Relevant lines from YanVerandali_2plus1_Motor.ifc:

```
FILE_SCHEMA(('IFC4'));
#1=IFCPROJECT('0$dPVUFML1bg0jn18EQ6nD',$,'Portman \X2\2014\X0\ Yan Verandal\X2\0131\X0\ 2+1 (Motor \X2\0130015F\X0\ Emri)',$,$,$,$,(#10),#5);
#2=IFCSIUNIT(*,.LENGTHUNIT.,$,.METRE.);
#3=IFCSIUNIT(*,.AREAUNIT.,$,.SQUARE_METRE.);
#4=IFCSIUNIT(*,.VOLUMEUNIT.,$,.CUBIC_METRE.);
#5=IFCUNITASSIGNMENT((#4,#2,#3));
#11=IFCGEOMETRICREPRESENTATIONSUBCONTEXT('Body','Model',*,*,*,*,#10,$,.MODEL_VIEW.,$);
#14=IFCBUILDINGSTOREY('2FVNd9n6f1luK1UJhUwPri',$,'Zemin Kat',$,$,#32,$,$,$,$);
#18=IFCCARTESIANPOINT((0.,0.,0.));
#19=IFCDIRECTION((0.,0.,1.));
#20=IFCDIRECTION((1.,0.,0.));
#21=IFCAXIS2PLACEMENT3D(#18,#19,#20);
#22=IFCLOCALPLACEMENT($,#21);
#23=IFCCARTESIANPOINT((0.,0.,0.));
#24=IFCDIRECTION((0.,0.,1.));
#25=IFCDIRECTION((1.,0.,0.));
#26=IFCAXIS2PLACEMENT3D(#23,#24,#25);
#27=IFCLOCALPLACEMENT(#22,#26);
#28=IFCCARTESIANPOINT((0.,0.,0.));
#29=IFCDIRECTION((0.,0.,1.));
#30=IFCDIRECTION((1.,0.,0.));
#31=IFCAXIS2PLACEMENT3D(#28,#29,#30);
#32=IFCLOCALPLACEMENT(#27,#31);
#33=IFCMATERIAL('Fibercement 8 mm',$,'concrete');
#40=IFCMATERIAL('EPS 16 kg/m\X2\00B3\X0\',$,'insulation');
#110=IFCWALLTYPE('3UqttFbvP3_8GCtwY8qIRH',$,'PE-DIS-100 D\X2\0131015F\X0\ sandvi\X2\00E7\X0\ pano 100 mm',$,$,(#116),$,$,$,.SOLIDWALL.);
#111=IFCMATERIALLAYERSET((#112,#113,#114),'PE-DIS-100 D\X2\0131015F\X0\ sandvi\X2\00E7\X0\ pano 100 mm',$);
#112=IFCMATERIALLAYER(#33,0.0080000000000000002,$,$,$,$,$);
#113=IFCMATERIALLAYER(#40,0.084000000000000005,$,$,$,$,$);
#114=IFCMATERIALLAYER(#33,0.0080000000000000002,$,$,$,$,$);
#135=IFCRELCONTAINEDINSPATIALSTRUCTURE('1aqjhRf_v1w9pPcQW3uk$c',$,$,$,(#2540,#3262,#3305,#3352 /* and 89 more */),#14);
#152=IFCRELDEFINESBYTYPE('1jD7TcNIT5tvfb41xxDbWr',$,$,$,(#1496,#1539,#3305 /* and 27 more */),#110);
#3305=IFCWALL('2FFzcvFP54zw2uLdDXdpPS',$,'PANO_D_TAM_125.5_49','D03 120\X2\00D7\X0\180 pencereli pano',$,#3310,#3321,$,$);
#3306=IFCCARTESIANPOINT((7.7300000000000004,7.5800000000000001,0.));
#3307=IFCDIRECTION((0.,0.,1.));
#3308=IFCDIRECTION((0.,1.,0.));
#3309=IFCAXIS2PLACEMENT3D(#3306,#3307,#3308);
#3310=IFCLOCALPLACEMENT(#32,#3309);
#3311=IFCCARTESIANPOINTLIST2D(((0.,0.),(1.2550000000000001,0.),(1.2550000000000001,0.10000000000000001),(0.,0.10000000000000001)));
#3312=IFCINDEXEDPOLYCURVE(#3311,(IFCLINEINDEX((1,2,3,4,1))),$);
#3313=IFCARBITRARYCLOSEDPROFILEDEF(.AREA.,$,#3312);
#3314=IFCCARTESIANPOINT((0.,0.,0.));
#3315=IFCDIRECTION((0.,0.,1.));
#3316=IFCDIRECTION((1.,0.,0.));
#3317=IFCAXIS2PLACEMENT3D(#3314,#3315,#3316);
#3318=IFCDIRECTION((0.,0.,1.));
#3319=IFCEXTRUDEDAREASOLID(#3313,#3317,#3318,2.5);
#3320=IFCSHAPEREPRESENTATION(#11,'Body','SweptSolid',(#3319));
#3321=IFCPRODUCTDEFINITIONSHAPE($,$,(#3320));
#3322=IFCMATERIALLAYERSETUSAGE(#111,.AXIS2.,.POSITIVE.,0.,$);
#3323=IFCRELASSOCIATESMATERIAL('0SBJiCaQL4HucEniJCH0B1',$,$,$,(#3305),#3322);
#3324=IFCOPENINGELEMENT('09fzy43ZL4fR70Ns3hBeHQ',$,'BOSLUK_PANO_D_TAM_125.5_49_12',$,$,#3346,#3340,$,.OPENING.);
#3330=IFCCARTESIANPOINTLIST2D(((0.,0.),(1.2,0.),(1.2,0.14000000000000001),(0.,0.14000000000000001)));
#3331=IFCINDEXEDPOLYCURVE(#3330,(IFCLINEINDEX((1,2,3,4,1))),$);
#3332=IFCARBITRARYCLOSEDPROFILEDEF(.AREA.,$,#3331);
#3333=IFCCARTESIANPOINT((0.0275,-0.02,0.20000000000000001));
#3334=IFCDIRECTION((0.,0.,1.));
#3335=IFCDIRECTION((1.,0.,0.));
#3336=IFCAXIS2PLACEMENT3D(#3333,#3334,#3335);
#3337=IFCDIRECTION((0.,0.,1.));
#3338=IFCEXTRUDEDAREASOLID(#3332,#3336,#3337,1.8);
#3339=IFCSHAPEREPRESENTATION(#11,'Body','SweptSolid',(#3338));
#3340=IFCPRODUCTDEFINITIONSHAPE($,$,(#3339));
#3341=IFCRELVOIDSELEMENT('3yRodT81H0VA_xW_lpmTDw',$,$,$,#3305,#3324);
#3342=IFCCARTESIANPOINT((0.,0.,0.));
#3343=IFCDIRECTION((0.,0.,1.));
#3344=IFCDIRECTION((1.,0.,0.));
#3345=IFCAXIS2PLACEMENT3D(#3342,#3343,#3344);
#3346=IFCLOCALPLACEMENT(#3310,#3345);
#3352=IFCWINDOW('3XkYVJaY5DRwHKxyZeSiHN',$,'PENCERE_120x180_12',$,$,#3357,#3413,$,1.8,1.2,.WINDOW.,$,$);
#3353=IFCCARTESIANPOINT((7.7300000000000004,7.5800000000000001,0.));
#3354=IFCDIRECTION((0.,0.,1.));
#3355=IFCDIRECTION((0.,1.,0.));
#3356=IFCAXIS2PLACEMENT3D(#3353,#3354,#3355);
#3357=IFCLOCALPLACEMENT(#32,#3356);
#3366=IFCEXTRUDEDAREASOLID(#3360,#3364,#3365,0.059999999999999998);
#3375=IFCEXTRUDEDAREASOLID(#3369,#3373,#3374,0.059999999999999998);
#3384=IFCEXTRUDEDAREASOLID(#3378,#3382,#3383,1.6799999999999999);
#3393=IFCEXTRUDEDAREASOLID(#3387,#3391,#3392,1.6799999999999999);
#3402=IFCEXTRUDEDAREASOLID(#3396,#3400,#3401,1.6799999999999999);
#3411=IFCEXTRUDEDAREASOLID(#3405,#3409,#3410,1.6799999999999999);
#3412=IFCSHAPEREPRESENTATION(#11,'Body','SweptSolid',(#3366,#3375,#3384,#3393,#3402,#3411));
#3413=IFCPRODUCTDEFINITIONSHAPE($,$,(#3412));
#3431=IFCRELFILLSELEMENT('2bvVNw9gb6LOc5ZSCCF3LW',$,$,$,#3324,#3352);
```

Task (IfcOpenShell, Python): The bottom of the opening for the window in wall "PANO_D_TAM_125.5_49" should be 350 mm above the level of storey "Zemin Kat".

```python
import numpy as np
import ifcopenshell
import ifcopenshell.api.geometry
import ifcopenshell.geom
import ifcopenshell.util.element
import ifcopenshell.util.placement
import ifcopenshell.util.shape
import ifcopenshell.util.unit

model = ifcopenshell.open("YanVerandali_2plus1_Motor.ifc")
unit_scale = ifcopenshell.util.unit.calculate_unit_scale(model)

window = model.by_guid("3XkYVJaY5DRwHKxyZeSiHN")
opening = window.FillsVoids[0].RelatingOpeningElement
storey = ifcopenshell.util.element.get_container(window, ifc_class="IfcBuildingStorey")
level = ifcopenshell.util.placement.get_local_placement(storey.ObjectPlacement)[2, 3]

# The opening's origin need not be at the sill, so measure its lowest point.
shape = ifcopenshell.geom.create_shape(ifcopenshell.geom.settings(), opening)
bottom = ifcopenshell.util.shape.get_shape_bottom_elevation(shape, shape.geometry) / unit_scale
dz = level + 0.35 / unit_scale - bottom

shift = np.array([0.0, 0.0, dz])
# The window is not placed relative to its opening, so move both.
for product in (opening, window):
    matrix = ifcopenshell.util.placement.get_local_placement(product.ObjectPlacement)
    matrix[:3, 3] += shift
    ifcopenshell.api.geometry.edit_object_placement(model, product=product, matrix=matrix, is_si=False)

print(f"moved by {dz * unit_scale:+.3f} m")

model.write("YanVerandali_2plus1_Motor-out.ifc")
```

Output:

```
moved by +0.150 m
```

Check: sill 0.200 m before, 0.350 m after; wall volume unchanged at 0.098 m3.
